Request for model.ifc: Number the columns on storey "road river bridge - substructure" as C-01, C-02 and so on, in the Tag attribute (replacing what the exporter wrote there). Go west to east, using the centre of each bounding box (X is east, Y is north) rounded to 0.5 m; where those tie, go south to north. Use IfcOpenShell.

First a look at what the model holds.

```python
import ifcopenshell
import ifcopenshell.util.element
import ifcopenshell.util.placement

model = ifcopenshell.open("model.ifc")
print(model.schema)
storey = next(s for s in model.by_type("IfcBuildingStorey") if s.Name == "road river bridge - substructure")
columns = [e for e in ifcopenshell.util.element.get_decomposition(storey) if e.is_a("IfcColumn")]
for e in sorted(columns, key=lambda e: e.id()):
    origin = ifcopenshell.util.placement.get_local_placement(e.ObjectPlacement)[:3, 3]
    print(e.id(), e.Tag, e.Name, origin.round(2) + 0.0, sep=" | ")
```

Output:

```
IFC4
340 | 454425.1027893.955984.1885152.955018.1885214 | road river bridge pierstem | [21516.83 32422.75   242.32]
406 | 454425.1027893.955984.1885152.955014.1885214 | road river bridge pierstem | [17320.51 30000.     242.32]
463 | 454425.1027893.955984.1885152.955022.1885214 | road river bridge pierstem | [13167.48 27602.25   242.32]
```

```python
import ifcopenshell
import ifcopenshell.geom
import ifcopenshell.util.element
import ifcopenshell.util.shape

model = ifcopenshell.open("model.ifc")
settings = ifcopenshell.geom.settings()
settings.set("use-world-coords", True)


def centre(element):
    shape = ifcopenshell.geom.create_shape(settings, element)
    return ifcopenshell.util.shape.get_bbox_centroid(shape.geometry)


storey = next(s for s in model.by_type("IfcBuildingStorey") if s.Name == "road river bridge - substructure")
columns = [e for e in ifcopenshell.util.element.get_decomposition(storey) if e.is_a("IfcColumn")]

# Insertion points can sit at a corner or the storey origin, so sort by the geometry (in metres).
centres = {e: centre(e) for e in columns}
columns.sort(key=lambda e: (round(centres[e][0] / 0.5), centres[e][1]))

for i, e in enumerate(columns, start=1):
    number = f"C-{i:02d}"
    e.Tag = number
    print(e.id(), number)

model.write("model_v2.ifc")
```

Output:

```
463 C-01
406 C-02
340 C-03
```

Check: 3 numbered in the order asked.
